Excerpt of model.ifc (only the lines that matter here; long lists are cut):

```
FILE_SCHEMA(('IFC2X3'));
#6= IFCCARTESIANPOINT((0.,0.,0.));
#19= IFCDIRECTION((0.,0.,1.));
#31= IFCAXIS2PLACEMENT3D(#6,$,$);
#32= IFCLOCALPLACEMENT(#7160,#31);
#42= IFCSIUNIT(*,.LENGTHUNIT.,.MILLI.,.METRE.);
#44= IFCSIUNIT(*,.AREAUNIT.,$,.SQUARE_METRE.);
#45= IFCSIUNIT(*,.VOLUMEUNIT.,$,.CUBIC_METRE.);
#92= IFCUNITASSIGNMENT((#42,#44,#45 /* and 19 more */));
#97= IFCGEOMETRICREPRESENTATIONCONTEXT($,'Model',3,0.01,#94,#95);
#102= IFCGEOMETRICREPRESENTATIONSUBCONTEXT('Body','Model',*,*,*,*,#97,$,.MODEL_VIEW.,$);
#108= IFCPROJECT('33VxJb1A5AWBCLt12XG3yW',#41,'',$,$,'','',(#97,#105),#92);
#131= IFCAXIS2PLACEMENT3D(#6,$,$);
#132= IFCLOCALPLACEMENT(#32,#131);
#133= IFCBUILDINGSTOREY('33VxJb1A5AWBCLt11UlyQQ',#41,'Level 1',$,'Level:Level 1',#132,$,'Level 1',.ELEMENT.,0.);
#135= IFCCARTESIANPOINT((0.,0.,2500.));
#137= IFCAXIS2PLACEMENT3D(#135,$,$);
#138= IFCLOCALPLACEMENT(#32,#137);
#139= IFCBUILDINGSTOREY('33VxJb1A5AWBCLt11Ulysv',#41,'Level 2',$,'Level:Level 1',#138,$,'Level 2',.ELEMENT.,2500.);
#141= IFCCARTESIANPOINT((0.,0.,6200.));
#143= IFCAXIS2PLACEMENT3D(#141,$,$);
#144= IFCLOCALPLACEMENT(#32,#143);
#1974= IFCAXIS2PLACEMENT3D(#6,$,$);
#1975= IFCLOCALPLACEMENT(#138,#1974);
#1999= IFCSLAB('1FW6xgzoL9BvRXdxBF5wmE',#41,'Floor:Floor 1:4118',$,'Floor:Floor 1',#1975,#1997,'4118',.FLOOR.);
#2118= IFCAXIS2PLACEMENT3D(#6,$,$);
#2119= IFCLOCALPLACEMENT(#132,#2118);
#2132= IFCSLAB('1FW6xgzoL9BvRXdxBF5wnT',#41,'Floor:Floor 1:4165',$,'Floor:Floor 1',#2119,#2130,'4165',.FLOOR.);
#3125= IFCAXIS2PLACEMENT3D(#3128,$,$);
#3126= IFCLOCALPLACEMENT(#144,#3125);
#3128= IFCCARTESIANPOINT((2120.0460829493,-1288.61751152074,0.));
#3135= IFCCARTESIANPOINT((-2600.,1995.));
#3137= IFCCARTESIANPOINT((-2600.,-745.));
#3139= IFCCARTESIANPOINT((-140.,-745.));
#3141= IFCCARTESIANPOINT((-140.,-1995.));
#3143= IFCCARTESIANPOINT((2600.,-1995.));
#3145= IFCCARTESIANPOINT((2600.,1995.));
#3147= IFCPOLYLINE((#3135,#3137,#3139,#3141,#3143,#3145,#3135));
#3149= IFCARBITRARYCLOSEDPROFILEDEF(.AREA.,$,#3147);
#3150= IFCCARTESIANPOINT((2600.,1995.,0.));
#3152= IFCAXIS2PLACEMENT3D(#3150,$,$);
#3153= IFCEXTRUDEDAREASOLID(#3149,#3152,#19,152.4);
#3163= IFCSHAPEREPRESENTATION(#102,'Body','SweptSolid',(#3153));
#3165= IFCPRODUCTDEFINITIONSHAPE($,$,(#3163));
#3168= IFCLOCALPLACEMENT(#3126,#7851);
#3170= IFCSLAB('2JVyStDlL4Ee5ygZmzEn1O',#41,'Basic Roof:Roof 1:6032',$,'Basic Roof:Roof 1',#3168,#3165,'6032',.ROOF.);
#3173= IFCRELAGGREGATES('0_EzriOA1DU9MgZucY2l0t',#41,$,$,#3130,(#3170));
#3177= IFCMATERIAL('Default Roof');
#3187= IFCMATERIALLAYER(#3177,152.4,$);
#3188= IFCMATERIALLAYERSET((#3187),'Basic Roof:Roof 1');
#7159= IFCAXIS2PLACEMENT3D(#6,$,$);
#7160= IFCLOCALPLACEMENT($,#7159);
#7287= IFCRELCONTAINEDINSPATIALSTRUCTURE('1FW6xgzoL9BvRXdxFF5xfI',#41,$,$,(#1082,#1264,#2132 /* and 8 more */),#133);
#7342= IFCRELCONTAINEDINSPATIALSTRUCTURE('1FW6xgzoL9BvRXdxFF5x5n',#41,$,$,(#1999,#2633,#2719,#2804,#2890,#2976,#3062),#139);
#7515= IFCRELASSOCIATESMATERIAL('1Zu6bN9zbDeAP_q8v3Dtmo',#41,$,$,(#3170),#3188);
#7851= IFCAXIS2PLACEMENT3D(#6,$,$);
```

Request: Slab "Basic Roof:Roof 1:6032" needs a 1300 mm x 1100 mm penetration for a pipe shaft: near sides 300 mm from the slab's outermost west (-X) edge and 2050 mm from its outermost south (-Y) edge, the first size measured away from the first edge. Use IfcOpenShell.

```python
import numpy as np
import ifcopenshell
import ifcopenshell.api.feature
import ifcopenshell.api.geometry
import ifcopenshell.api.root
import ifcopenshell.geom
import ifcopenshell.util.placement
import ifcopenshell.util.representation
import ifcopenshell.util.shape
import ifcopenshell.util.unit

model = ifcopenshell.open("model.ifc")
unit_scale = ifcopenshell.util.unit.calculate_unit_scale(model)
settings = ifcopenshell.geom.settings()


def volume(element):
    """Net volume in cubic metres, openings subtracted."""
    shape = ifcopenshell.geom.create_shape(settings, element)
    return ifcopenshell.util.shape.get_volume(shape.geometry)


slab = model.by_guid("2JVyStDlL4Ee5ygZmzEn1O")
before = volume(slab)

# Extent in the slab's own axes, in metres. The edges named are its -X and -Y sides.
slab_shape = ifcopenshell.geom.create_shape(settings, slab)
vertices = ifcopenshell.util.shape.get_vertices(slab_shape.geometry)
x_min, y_min, bottom = vertices.min(axis=0)
top = vertices[:, 2].max()

opening = ifcopenshell.api.root.create_entity(model, ifc_class="IfcOpeningElement", name="Pipe shaft opening")
context = ifcopenshell.util.representation.get_context(model, "Model", "Body", "MODEL_VIEW")
width, depth = 1.3, 1.1
outline = [(0.0, 0.0), (width, 0.0), (width, depth), (0.0, depth), (0.0, 0.0)]
# Overshoot both faces by 50 mm so the cut is clean.
shape = ifcopenshell.api.geometry.add_slab_representation(
    model, context=context, depth=top - bottom + 0.1, polyline=outline
)
ifcopenshell.api.geometry.assign_representation(model, product=opening, representation=shape)

matrix = ifcopenshell.util.placement.get_local_placement(slab.ObjectPlacement)
matrix[:, 3] = matrix @ np.append(np.array([x_min + 0.3, y_min + 2.05, bottom - 0.05]) / unit_scale, 1.0)
ifcopenshell.api.geometry.edit_object_placement(model, product=opening, matrix=matrix, is_si=False)
ifcopenshell.api.feature.add_feature(model, feature=opening, element=slab)

after = volume(slab)

print(f"slab volume {before:.3f} -> {after:.3f} m3")

model.write("model_updated.ifc")
```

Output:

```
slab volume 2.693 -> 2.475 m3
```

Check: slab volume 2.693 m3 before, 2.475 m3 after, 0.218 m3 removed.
